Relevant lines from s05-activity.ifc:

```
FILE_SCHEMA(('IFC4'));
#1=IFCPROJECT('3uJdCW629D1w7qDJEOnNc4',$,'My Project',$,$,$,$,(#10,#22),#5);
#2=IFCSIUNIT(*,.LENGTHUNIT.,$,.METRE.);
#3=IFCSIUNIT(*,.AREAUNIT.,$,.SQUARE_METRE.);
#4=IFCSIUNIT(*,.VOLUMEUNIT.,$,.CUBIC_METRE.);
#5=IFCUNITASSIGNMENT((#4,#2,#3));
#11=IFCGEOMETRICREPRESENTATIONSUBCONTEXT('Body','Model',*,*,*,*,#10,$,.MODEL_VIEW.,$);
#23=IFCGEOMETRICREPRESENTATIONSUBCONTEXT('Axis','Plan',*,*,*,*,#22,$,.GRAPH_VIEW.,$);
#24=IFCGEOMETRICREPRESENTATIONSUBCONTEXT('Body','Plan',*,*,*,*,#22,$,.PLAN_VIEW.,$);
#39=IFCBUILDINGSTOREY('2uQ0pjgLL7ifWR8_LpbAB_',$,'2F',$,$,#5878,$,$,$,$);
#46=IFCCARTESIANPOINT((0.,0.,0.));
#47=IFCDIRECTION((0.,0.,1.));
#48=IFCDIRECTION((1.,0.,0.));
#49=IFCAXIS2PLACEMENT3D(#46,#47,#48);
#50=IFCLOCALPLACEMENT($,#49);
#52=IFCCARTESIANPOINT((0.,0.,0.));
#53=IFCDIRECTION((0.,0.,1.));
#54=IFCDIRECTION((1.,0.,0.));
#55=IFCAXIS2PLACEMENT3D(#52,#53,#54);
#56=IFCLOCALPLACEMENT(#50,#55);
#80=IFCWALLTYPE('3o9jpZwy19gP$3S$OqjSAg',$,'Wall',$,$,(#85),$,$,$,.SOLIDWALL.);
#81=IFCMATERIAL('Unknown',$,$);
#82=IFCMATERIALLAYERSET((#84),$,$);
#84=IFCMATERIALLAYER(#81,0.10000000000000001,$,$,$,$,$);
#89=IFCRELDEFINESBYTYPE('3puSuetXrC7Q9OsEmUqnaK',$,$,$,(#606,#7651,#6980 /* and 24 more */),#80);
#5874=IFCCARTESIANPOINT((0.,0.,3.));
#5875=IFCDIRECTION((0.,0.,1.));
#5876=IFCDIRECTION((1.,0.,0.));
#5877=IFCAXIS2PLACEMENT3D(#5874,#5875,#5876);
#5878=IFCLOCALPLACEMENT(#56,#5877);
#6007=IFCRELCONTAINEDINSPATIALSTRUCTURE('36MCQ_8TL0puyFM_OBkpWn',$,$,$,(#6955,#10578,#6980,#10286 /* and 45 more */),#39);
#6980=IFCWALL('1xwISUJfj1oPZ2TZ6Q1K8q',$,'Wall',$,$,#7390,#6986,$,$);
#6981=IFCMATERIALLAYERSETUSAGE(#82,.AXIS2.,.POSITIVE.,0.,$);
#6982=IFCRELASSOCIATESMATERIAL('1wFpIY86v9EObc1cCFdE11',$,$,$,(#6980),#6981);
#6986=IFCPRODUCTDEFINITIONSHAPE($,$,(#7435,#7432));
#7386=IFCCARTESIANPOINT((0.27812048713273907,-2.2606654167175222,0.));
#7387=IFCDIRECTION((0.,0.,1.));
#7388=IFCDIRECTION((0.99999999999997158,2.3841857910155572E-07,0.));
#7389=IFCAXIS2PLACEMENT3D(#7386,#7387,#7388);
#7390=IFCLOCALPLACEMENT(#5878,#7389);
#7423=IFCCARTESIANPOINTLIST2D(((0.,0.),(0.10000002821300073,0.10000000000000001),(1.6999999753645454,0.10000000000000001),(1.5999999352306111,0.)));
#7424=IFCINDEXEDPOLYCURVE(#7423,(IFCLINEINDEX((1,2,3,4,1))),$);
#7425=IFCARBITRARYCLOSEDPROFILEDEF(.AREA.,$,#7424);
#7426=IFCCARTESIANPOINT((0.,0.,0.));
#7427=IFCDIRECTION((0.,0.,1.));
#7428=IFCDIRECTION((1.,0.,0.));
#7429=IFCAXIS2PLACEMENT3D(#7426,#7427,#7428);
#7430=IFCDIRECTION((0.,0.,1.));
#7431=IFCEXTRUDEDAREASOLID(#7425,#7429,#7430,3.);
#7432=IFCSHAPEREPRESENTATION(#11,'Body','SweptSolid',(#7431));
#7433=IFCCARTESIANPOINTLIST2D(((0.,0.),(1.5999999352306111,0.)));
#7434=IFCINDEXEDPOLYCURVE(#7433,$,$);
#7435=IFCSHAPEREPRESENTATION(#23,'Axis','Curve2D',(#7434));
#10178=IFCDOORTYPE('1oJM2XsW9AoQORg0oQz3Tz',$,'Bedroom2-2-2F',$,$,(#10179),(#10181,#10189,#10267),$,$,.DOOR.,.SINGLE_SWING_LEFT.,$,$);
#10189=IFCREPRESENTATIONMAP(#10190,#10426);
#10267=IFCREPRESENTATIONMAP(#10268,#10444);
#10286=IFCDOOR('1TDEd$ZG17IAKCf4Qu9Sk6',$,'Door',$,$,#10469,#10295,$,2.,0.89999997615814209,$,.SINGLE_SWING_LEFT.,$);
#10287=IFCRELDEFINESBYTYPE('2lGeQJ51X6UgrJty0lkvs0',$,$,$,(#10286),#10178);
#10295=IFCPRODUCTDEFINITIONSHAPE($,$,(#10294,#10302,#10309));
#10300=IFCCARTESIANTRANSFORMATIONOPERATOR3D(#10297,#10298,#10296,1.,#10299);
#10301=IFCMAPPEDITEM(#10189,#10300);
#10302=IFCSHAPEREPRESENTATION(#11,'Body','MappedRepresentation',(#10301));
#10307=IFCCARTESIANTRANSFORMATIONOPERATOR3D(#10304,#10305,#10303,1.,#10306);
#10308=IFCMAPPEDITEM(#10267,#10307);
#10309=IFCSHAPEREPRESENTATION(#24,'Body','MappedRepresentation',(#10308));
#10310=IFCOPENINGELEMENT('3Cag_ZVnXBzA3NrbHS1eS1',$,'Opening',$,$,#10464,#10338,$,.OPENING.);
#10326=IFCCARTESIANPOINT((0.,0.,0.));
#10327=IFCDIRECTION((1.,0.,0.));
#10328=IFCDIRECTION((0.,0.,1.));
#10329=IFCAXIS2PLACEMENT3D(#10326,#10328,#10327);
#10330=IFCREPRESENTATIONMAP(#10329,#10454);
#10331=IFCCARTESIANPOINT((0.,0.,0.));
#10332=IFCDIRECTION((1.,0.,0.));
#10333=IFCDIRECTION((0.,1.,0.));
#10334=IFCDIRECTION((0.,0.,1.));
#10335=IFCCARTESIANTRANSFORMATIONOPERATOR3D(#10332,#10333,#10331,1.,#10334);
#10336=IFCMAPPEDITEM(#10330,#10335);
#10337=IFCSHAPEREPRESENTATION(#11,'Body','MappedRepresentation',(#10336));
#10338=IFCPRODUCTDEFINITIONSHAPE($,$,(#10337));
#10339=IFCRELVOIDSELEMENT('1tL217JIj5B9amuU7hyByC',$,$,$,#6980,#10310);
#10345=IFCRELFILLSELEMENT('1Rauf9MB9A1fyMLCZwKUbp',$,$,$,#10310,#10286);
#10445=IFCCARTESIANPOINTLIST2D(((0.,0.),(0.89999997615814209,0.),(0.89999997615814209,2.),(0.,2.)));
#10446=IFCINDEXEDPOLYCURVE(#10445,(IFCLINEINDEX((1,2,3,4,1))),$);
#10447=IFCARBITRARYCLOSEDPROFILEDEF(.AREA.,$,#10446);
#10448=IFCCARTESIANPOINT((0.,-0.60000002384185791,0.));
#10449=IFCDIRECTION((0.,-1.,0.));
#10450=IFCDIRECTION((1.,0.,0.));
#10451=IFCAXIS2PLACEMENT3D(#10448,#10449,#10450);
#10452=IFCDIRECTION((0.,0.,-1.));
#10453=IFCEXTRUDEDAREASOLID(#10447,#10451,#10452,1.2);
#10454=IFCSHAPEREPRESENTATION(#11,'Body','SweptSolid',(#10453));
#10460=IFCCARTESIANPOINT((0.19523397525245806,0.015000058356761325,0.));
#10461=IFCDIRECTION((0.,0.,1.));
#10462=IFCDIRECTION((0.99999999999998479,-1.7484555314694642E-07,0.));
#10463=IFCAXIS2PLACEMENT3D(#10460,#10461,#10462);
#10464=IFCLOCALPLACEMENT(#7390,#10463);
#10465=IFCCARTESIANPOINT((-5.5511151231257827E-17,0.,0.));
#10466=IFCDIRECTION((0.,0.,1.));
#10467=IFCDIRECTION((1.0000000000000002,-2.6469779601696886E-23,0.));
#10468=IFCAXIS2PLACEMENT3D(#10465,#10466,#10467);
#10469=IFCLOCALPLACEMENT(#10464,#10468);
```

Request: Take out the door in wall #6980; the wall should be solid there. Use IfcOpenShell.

```python
import ifcopenshell
import ifcopenshell.api.feature
import ifcopenshell.api.root
import ifcopenshell.geom
import ifcopenshell.util.shape

model = ifcopenshell.open("s05-activity.ifc")
settings = ifcopenshell.geom.settings()


def volume(element):
    """Net volume in cubic metres, openings subtracted."""
    shape = ifcopenshell.geom.create_shape(settings, element)
    return ifcopenshell.util.shape.get_volume(shape.geometry)


door = model.by_guid("1TDEd$ZG17IAKCf4Qu9Sk6")
opening = door.FillsVoids[0].RelatingOpeningElement
wall = opening.VoidsElements[0].RelatingBuildingElement
before = volume(wall)

ifcopenshell.api.root.remove_product(model, product=door)
ifcopenshell.api.feature.remove_feature(model, feature=opening)

after = volume(wall)

print(f"wall volume {before:.3f} -> {after:.3f} m3")

model.write("s05-activity_v2.ifc")
```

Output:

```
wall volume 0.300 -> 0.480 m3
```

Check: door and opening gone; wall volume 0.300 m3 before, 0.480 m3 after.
